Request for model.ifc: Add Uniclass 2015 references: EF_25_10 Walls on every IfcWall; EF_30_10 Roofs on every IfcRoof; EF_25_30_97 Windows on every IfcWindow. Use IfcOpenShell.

First a look at what the model holds.

```python
import ifcopenshell

model = ifcopenshell.open("model.ifc")
print(model.schema)
print("classifications:", [c.Name for c in model.by_type("IfcClassification")])
for ifc_class in ("IfcDoor", "IfcRoof", "IfcStair", "IfcWall", "IfcWindow"):
    print(ifc_class, len(model.by_type(ifc_class)))
```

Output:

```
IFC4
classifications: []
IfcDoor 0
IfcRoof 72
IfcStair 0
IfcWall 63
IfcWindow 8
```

```python
import ifcopenshell
import ifcopenshell.api.classification

model = ifcopenshell.open("model.ifc")

system = ifcopenshell.api.classification.add_classification(model, classification="Uniclass 2015")

codes = {
    "IfcWall": ("EF_25_10", "Walls"),
    "IfcRoof": ("EF_30_10", "Roofs"),
    "IfcWindow": ("EF_25_30_97", "Windows"),
}
for ifc_class, (code, name) in codes.items():
    products = model.by_type(ifc_class)
    ifcopenshell.api.classification.add_reference(
        model, products=products, classification=system, identification=code, name=name
    )
    print(code, len(products))

model.write("model_rev.ifc")
```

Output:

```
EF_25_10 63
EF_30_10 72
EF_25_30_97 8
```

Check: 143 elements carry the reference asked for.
